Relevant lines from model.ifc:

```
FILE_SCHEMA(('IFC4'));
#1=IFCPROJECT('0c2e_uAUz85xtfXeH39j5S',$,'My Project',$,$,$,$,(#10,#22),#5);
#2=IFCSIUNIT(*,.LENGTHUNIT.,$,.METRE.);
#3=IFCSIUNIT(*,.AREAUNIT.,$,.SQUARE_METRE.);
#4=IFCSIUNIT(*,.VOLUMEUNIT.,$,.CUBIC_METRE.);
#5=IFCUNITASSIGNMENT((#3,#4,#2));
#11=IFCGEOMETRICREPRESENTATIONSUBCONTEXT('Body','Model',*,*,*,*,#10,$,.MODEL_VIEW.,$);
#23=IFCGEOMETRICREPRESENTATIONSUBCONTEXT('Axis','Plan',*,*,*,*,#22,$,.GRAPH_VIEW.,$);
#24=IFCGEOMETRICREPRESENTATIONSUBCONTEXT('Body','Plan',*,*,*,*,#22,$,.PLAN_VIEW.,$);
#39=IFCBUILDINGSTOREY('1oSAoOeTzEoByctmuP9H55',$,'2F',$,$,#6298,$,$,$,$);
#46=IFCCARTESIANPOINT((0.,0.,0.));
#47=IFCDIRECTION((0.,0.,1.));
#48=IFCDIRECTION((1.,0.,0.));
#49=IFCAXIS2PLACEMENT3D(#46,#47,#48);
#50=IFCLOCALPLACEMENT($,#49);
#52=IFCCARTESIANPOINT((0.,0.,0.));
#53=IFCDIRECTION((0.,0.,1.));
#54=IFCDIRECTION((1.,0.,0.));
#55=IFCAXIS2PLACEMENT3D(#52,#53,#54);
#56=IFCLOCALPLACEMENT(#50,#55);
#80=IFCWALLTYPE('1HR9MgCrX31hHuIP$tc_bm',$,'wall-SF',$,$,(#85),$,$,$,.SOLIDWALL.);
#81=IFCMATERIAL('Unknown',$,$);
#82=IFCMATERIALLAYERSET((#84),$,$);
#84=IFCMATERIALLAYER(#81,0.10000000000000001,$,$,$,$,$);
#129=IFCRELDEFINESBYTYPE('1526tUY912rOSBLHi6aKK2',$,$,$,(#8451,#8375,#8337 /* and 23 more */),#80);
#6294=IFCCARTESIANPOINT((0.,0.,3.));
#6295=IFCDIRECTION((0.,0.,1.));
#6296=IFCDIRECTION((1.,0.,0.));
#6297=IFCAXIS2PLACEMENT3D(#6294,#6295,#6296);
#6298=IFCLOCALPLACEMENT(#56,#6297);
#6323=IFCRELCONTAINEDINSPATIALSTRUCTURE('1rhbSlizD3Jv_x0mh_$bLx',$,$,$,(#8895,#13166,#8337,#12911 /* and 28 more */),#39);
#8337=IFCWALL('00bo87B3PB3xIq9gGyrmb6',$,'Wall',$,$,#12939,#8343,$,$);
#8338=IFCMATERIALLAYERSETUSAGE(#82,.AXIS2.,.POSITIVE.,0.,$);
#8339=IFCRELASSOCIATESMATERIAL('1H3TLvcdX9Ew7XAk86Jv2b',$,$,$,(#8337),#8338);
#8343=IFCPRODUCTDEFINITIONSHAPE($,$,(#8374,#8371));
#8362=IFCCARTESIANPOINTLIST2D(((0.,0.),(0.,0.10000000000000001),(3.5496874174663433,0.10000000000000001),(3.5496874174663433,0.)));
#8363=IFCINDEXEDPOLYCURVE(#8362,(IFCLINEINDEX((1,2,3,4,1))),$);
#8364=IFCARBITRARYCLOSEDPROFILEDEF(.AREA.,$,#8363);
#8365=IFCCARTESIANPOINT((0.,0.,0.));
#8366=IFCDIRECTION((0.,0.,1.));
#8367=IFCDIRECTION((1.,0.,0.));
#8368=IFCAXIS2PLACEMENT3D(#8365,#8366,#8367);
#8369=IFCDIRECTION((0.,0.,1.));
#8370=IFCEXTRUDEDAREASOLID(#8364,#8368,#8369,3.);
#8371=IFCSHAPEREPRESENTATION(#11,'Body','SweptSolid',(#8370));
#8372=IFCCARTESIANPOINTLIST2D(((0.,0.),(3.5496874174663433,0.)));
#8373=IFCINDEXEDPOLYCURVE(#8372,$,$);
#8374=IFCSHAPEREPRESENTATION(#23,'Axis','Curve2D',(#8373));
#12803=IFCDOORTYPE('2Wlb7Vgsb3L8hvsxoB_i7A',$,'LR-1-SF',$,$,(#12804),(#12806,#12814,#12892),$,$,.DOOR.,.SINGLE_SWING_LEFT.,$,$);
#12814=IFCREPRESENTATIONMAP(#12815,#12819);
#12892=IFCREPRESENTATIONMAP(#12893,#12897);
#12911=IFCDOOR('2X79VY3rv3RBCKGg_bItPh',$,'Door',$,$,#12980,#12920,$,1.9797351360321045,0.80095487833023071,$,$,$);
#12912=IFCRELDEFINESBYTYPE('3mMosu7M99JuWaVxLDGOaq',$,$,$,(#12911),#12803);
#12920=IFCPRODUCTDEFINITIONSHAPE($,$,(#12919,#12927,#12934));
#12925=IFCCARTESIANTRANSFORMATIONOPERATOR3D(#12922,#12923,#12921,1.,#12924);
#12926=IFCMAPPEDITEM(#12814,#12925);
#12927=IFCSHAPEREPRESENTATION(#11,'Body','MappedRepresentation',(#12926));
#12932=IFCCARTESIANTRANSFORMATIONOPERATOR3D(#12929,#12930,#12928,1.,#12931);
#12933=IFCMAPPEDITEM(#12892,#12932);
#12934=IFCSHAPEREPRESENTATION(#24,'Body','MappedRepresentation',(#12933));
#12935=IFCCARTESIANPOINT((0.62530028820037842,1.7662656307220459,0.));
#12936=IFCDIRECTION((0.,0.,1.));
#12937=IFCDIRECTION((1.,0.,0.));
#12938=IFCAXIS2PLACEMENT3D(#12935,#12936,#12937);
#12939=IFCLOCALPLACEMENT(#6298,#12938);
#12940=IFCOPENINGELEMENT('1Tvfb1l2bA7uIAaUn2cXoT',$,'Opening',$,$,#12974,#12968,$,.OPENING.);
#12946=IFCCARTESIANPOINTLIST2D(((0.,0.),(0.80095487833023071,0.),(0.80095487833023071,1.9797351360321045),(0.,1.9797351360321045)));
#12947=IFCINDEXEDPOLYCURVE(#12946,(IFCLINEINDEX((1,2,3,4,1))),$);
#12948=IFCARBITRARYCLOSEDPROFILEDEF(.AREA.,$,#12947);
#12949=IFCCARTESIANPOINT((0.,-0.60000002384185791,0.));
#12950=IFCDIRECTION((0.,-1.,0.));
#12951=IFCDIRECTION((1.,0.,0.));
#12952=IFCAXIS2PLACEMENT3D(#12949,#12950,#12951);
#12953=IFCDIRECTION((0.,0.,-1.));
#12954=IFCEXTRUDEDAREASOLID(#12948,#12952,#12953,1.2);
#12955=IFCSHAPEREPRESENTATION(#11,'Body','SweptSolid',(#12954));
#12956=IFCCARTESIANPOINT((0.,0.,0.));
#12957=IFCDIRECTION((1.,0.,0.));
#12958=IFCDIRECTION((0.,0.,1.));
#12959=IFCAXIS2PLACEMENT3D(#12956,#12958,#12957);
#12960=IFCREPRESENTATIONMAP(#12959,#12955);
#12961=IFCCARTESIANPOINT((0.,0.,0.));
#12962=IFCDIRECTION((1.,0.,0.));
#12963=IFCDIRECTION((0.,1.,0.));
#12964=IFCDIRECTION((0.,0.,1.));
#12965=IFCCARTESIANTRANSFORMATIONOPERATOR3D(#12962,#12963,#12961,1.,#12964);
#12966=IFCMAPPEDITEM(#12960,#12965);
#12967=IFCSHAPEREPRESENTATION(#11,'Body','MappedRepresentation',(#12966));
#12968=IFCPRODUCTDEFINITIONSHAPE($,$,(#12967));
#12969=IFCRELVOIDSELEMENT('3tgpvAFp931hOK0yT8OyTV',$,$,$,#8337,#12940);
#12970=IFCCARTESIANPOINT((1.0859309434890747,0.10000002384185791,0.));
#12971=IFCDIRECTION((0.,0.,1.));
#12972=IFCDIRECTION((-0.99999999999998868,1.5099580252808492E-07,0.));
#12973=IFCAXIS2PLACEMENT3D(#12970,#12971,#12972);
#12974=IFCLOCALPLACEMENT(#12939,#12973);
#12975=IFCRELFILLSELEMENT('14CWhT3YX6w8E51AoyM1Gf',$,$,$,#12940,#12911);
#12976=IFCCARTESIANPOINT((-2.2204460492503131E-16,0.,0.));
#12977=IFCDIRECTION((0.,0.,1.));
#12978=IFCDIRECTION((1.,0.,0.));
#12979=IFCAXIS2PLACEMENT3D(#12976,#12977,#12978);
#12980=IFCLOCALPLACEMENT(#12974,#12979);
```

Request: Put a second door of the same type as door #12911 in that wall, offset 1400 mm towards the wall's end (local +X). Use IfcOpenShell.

```python
import ifcopenshell
import ifcopenshell.api.feature
import ifcopenshell.api.geometry
import ifcopenshell.api.root
import ifcopenshell.geom
import ifcopenshell.util.element
import ifcopenshell.util.placement
import ifcopenshell.util.shape

model = ifcopenshell.open("model.ifc")
settings = ifcopenshell.geom.settings()


def volume(element):
    """Net volume in cubic metres, openings subtracted."""
    shape = ifcopenshell.geom.create_shape(settings, element)
    return ifcopenshell.util.shape.get_volume(shape.geometry)


door = model.by_id(12911)
opening = door.FillsVoids[0].RelatingOpeningElement
wall = opening.VoidsElements[0].RelatingBuildingElement
before = volume(wall)
shift = ifcopenshell.util.placement.get_local_placement(wall.ObjectPlacement)[:3, 0] * 1.4

# copy_class copies the void relationship, type, container and properties, but no geometry.
new_opening = ifcopenshell.api.root.copy_class(model, product=opening)
new_opening.Representation = ifcopenshell.util.element.copy_deep(
    model, opening.Representation, exclude=["IfcGeometricRepresentationContext", "IfcRepresentationMap"]
)
new_door = ifcopenshell.api.root.copy_class(model, product=door)
new_door.Representation = ifcopenshell.util.element.copy_deep(
    model, door.Representation, exclude=["IfcGeometricRepresentationContext", "IfcRepresentationMap"]
)
ifcopenshell.api.feature.add_filling(model, opening=new_opening, element=new_door)

for old, new in ((opening, new_opening), (door, new_door)):
    matrix = ifcopenshell.util.placement.get_local_placement(old.ObjectPlacement)
    matrix[:3, 3] += shift
    ifcopenshell.api.geometry.edit_object_placement(model, product=new, matrix=matrix, is_si=False)

after = volume(wall)

print(f"wall volume {before:.3f} -> {after:.3f} m3")

model.write("model_edited.ifc")
```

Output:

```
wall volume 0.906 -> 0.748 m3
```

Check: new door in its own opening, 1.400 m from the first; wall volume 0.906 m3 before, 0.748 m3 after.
